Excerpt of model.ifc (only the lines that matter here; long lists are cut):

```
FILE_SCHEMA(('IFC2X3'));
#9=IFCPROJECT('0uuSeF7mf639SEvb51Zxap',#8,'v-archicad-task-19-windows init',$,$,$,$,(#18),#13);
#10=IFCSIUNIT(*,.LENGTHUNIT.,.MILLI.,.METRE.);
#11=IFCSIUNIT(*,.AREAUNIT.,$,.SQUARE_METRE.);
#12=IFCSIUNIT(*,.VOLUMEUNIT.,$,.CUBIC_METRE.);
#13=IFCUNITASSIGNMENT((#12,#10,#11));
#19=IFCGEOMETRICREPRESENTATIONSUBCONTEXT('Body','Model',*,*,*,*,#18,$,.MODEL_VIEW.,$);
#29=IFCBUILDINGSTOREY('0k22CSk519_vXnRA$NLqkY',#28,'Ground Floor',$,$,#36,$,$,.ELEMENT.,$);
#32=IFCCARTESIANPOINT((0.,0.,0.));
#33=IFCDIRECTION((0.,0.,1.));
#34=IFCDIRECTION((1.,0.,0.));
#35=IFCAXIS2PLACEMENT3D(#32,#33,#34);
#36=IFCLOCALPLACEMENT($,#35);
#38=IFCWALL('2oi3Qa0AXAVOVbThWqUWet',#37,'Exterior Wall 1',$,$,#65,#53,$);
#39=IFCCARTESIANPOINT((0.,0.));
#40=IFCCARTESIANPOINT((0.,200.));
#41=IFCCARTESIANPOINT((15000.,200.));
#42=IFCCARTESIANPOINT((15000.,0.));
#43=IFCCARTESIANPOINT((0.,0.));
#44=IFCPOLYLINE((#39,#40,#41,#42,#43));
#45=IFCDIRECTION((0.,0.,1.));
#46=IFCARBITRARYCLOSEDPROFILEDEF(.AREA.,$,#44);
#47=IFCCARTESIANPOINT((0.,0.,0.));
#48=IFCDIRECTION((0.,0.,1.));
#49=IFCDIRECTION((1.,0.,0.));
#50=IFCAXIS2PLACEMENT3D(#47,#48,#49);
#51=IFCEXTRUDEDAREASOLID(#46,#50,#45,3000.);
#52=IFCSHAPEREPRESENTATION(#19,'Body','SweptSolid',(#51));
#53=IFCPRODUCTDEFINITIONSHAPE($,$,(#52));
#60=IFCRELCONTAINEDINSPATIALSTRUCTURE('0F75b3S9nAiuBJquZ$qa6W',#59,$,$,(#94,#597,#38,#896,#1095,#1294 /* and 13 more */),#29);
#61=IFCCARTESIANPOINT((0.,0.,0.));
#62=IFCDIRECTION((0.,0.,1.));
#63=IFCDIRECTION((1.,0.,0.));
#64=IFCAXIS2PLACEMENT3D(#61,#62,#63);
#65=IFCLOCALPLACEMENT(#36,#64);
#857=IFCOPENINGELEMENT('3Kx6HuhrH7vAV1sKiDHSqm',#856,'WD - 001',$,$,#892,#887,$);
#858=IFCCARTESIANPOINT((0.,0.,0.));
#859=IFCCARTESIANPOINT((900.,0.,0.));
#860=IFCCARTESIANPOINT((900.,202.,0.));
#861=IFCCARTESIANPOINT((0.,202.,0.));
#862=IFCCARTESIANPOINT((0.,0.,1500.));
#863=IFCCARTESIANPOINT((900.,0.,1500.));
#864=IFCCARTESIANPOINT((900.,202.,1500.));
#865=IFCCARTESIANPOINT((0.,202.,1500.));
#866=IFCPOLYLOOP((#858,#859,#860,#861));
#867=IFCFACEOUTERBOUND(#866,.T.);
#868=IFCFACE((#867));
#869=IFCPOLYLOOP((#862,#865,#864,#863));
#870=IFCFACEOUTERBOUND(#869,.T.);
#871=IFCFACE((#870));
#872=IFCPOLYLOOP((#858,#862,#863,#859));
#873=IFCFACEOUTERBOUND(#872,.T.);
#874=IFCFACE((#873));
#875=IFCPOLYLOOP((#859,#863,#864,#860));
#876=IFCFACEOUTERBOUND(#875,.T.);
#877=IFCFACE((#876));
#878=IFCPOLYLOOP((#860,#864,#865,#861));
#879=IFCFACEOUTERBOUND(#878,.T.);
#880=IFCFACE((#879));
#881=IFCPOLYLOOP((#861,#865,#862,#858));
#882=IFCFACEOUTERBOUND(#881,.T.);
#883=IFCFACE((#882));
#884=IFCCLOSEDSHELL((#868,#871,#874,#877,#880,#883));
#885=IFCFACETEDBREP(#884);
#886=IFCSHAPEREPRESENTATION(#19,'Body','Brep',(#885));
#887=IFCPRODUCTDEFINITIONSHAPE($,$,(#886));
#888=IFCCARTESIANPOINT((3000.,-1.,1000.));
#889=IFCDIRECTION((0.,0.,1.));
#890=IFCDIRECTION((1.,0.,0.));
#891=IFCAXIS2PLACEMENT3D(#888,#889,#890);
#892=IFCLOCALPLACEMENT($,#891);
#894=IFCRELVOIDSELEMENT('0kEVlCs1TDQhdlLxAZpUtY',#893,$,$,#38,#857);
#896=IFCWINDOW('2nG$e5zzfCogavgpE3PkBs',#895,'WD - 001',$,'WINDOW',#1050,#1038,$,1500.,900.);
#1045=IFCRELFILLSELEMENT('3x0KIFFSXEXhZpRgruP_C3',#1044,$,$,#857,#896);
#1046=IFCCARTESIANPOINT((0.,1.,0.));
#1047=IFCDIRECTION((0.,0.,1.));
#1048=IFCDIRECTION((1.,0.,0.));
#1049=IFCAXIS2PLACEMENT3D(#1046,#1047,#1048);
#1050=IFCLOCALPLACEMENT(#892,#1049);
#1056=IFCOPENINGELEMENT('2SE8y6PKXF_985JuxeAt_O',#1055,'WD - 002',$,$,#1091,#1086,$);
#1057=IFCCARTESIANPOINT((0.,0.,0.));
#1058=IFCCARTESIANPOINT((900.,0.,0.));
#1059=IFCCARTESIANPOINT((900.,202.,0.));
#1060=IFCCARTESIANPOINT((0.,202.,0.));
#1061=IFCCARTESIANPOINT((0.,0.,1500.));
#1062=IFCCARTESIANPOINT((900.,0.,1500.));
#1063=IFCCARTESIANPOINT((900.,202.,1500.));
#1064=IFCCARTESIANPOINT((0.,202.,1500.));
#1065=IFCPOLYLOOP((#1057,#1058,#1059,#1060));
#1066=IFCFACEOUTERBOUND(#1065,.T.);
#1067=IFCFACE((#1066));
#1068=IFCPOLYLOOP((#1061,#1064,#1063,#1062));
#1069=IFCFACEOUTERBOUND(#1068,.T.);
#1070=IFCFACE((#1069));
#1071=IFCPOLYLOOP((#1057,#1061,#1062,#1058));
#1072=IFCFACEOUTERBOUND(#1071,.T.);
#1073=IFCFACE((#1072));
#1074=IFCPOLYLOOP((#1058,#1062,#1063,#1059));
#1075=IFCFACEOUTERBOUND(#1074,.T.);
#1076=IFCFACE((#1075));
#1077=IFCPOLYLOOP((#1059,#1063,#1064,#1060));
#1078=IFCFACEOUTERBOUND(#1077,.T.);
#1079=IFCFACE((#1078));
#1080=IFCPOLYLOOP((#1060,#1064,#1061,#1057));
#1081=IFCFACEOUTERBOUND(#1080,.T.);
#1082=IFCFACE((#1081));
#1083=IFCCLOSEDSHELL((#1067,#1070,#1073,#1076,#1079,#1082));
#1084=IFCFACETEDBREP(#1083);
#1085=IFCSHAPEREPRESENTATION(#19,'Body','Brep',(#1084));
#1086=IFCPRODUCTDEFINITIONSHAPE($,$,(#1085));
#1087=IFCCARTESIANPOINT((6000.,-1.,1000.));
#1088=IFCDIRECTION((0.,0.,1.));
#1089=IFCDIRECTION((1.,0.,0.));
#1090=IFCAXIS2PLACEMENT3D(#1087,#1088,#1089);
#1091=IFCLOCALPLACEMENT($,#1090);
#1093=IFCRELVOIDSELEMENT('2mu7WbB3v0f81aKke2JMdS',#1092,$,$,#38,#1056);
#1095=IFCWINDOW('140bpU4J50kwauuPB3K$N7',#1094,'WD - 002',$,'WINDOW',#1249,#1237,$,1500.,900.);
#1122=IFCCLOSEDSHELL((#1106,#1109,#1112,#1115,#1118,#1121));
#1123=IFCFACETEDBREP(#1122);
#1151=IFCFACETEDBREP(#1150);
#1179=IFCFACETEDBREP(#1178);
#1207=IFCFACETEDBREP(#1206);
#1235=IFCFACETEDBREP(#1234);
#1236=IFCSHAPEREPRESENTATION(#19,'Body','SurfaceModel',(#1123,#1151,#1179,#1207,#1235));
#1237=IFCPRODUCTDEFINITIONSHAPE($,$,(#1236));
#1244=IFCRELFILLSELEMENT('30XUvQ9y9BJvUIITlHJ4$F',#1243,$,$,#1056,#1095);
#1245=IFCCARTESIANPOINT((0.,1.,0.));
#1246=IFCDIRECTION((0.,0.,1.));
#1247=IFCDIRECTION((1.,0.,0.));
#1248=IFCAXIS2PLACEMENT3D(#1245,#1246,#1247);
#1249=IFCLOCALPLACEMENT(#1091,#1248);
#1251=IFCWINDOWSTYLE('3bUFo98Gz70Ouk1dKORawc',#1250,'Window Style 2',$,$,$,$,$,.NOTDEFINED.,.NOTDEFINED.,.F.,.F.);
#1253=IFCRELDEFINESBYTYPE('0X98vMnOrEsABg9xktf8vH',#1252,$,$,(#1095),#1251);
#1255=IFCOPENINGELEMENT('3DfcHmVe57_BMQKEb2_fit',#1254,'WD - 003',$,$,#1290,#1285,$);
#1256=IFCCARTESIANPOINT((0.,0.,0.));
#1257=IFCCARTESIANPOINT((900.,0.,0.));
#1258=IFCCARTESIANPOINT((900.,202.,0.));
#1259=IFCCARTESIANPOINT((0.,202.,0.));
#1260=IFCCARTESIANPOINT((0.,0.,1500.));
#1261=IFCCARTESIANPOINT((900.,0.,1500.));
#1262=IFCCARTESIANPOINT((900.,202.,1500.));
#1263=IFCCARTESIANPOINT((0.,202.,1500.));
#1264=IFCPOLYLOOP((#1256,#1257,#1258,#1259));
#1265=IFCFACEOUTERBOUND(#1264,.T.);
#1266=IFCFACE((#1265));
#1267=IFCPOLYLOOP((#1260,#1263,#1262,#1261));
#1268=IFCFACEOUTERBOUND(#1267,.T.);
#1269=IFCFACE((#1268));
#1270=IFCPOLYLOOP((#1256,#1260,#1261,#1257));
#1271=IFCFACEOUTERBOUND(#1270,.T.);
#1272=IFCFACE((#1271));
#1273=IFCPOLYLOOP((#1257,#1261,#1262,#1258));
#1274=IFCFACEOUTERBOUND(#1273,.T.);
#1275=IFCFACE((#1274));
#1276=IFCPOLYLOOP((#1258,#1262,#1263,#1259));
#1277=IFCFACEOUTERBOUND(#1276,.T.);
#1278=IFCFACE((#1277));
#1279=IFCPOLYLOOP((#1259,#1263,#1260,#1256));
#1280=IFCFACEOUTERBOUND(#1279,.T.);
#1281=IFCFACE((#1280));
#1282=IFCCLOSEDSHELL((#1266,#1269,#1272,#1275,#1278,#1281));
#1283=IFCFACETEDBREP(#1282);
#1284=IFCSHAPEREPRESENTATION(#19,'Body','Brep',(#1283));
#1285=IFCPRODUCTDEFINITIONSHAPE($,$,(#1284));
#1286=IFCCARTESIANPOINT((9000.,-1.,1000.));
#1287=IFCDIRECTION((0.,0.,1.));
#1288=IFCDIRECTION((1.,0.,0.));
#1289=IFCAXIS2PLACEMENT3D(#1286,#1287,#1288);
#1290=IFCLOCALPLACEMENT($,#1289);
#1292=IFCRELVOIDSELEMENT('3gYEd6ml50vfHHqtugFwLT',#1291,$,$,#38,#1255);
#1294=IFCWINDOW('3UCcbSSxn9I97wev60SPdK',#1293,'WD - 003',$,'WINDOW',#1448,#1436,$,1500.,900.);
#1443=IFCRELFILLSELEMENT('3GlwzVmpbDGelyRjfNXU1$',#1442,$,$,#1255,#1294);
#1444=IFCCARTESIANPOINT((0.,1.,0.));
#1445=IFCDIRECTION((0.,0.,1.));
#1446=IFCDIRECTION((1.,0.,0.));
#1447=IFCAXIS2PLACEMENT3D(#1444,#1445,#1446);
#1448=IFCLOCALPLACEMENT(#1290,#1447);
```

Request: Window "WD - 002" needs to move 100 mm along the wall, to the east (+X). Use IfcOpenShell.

```python
import ifcopenshell
import ifcopenshell.api.geometry
import ifcopenshell.util.placement

model = ifcopenshell.open("model.ifc")

window = model.by_id(1095)
opening = window.FillsVoids[0].RelatingOpeningElement
wall = opening.VoidsElements[0].RelatingBuildingElement

wall_matrix = ifcopenshell.util.placement.get_local_placement(wall.ObjectPlacement)
shift = wall_matrix[:3, 0] * 100.0
before = ifcopenshell.util.placement.get_local_placement(window.ObjectPlacement)[:3, 3].copy()

# The window is placed relative to its opening, so it follows when the opening moves.
matrix = ifcopenshell.util.placement.get_local_placement(opening.ObjectPlacement)
matrix[:3, 3] += shift
ifcopenshell.api.geometry.edit_object_placement(
    model, product=opening, matrix=matrix, is_si=False, should_transform_children=True
)

after = ifcopenshell.util.placement.get_local_placement(window.ObjectPlacement)[:3, 3]
print("window moved by", (after - before).round(3) + 0.0)

model.write("model_rev.ifc")
```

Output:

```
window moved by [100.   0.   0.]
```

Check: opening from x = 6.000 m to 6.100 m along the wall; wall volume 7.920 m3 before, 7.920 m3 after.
